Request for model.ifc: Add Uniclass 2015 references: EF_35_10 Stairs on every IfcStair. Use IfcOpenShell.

First a look at what the model holds.

```python
import ifcopenshell

model = ifcopenshell.open("model.ifc")
print(model.schema)
print("classifications:", [c.Name for c in model.by_type("IfcClassification")])
for ifc_class in ("IfcDoor", "IfcRoof", "IfcStair", "IfcWall", "IfcWindow"):
    print(ifc_class, len(model.by_type(ifc_class)))
```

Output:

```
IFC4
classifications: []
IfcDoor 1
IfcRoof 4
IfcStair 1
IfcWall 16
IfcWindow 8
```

```python
import ifcopenshell
import ifcopenshell.api.classification

model = ifcopenshell.open("model.ifc")

system = ifcopenshell.api.classification.add_classification(model, classification="Uniclass 2015")

codes = {
    "IfcStair": ("EF_35_10", "Stairs"),
}
for ifc_class, (code, name) in codes.items():
    products = model.by_type(ifc_class)
    ifcopenshell.api.classification.add_reference(
        model, products=products, classification=system, identification=code, name=name
    )
    print(code, len(products))

model.write("model-out.ifc")
```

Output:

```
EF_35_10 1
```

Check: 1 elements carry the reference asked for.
